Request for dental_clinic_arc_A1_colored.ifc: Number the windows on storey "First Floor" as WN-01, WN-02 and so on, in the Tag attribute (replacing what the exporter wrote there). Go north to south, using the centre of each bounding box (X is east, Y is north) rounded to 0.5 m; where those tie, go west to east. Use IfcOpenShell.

First a look at what the model holds.

```python
import ifcopenshell
import ifcopenshell.util.element
import ifcopenshell.util.placement

model = ifcopenshell.open("dental_clinic_arc_A1_colored.ifc")
print(model.schema)
storey = next(s for s in model.by_type("IfcBuildingStorey") if s.Name == "First Floor")
windows = [e for e in ifcopenshell.util.element.get_decomposition(storey) if e.is_a("IfcWindow")]
for e in sorted(windows, key=lambda e: e.id()):
    origin = ifcopenshell.util.placement.get_local_placement(e.ObjectPlacement)[:3, 3]
    print(e.id(), e.Tag, e.Name, origin.round(2) + 0.0, sep=" | ")
```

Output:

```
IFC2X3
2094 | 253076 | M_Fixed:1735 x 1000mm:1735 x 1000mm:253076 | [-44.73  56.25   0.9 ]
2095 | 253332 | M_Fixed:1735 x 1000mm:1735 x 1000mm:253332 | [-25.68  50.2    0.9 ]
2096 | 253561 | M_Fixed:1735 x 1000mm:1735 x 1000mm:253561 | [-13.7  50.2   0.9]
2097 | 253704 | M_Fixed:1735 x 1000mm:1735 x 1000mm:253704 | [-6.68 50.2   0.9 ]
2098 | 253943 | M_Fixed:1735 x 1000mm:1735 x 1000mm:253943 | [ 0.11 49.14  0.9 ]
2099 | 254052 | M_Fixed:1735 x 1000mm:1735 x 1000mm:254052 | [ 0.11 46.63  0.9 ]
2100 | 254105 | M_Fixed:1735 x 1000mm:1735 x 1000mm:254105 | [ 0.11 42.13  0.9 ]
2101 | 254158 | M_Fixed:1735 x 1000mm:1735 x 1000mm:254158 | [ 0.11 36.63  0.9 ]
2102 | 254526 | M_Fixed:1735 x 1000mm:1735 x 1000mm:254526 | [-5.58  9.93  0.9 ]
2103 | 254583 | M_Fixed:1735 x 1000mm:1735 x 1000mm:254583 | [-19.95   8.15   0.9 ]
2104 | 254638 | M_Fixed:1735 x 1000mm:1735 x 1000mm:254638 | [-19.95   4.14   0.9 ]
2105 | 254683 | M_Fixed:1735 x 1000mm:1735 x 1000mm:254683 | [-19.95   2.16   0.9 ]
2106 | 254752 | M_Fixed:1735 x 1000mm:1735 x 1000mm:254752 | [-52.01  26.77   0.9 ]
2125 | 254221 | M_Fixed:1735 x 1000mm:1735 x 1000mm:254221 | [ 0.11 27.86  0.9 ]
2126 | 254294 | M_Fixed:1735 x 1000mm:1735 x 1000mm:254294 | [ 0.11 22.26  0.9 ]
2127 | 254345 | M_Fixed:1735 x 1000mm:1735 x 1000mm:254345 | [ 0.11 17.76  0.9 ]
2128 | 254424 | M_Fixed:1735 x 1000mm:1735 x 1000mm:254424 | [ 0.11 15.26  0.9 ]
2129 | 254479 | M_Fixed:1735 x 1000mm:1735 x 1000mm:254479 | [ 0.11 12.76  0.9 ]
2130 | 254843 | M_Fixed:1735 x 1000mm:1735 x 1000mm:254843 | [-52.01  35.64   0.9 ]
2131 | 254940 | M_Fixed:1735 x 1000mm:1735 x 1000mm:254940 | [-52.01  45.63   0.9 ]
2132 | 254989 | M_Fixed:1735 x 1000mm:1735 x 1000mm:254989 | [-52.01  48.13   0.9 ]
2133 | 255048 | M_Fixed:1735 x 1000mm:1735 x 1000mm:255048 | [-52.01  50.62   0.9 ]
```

```python
import ifcopenshell
import ifcopenshell.geom
import ifcopenshell.util.element
import ifcopenshell.util.shape

model = ifcopenshell.open("dental_clinic_arc_A1_colored.ifc")
settings = ifcopenshell.geom.settings()
settings.set("use-world-coords", True)


def centre(element):
    shape = ifcopenshell.geom.create_shape(settings, element)
    return ifcopenshell.util.shape.get_bbox_centroid(shape.geometry)


storey = next(s for s in model.by_type("IfcBuildingStorey") if s.Name == "First Floor")
windows = [e for e in ifcopenshell.util.element.get_decomposition(storey) if e.is_a("IfcWindow")]

# Insertion points can sit at a corner or the storey origin, so sort by the geometry (in metres).
centres = {e: centre(e) for e in windows}
windows.sort(key=lambda e: (-round(centres[e][1] / 0.5), centres[e][0]))

for i, e in enumerate(windows, start=1):
    number = f"WN-{i:02d}"
    e.Tag = number
    print(e.id(), number)

model.write("dental_clinic_arc_A1_colored_v2.ifc")
```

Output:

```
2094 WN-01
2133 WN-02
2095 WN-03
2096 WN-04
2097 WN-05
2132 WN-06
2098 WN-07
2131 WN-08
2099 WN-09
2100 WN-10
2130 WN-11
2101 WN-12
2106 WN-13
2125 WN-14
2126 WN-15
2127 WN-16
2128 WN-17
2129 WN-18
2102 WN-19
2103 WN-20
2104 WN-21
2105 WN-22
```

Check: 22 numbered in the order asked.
